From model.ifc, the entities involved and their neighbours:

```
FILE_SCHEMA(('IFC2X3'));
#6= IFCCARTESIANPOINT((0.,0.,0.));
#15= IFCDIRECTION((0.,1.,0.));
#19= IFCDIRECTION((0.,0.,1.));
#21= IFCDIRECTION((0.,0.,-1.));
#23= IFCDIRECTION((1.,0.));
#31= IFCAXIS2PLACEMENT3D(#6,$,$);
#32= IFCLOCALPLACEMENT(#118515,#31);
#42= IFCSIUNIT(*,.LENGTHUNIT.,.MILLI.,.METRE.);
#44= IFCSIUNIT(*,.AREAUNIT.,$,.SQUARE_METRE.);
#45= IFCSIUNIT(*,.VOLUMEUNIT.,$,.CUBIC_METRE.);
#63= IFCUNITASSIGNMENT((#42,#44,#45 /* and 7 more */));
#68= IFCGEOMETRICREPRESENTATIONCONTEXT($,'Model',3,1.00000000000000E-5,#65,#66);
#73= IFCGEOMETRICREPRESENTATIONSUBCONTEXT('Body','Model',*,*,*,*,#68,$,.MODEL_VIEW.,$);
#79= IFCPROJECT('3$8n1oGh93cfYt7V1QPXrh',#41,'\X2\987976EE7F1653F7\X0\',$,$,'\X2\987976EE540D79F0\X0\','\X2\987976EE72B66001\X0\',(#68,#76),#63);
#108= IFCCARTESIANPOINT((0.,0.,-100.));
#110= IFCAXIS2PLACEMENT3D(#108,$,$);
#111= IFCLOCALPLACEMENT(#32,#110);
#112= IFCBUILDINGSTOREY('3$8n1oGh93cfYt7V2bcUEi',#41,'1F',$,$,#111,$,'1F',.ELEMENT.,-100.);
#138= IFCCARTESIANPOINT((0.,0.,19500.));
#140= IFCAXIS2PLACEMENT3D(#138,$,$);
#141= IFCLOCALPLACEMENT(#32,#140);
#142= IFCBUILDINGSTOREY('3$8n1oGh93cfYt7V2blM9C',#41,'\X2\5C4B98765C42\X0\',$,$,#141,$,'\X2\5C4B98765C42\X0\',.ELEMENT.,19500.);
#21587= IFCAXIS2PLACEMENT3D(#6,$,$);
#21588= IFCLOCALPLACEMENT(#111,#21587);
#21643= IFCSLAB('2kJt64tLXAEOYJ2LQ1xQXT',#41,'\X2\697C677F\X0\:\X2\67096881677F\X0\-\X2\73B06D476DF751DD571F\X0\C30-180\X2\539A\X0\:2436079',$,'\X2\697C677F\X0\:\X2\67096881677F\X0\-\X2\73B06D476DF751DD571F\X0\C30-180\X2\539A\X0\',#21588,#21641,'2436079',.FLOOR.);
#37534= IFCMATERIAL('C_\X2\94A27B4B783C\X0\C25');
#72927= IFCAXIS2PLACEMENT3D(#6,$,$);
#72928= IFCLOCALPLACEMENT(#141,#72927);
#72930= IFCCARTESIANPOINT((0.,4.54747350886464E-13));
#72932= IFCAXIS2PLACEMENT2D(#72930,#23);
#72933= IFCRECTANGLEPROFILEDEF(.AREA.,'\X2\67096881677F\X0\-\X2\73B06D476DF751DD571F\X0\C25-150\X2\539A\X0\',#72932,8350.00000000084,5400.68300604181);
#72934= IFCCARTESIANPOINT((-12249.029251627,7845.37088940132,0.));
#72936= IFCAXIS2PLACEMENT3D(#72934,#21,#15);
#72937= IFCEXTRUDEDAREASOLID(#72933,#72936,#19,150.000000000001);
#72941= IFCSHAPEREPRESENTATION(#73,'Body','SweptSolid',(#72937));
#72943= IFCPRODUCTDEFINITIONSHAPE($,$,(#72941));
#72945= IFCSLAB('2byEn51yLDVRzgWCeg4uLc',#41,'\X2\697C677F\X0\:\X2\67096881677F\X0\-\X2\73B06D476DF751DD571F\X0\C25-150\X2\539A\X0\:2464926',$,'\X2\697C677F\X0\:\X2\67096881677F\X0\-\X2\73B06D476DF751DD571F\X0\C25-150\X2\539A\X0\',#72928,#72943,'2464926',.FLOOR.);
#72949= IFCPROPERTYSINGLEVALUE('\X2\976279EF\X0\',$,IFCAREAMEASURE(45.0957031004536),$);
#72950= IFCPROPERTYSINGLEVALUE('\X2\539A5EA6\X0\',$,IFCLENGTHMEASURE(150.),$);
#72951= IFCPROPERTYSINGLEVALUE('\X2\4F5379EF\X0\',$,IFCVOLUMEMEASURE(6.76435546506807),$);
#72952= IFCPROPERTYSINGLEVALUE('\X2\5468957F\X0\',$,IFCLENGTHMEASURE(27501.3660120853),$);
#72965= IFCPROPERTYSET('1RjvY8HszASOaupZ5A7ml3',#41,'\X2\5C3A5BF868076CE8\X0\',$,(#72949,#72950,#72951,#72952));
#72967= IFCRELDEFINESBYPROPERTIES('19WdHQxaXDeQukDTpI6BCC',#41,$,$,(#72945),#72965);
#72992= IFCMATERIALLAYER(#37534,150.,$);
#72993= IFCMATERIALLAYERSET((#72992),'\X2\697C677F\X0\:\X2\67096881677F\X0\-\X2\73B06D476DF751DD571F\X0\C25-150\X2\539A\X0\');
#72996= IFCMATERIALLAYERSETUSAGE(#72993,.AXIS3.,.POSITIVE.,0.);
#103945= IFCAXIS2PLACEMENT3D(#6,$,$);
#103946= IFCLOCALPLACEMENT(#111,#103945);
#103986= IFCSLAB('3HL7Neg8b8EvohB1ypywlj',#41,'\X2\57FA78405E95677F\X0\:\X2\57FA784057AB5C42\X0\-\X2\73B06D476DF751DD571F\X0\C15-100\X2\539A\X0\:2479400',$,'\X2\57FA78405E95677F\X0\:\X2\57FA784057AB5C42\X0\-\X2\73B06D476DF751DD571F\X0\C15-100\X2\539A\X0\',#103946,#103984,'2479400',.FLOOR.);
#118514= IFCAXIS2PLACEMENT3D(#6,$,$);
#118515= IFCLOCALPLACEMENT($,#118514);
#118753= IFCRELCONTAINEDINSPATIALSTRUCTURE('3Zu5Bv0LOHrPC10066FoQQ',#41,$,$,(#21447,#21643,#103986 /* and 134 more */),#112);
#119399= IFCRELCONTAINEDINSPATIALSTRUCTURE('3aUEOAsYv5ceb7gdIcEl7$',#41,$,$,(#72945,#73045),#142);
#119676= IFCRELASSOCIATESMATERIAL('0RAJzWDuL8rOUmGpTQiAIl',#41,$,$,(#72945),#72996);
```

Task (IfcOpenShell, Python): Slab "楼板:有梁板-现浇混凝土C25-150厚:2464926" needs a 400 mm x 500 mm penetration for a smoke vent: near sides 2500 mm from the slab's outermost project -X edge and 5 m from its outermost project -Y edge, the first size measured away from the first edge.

```python
import numpy as np
import ifcopenshell
import ifcopenshell.api.feature
import ifcopenshell.api.geometry
import ifcopenshell.api.pset
import ifcopenshell.api.root
import ifcopenshell.geom
import ifcopenshell.util.element
import ifcopenshell.util.placement
import ifcopenshell.util.representation
import ifcopenshell.util.shape
import ifcopenshell.util.unit

model = ifcopenshell.open("model.ifc")
unit_scale = ifcopenshell.util.unit.calculate_unit_scale(model)
area_scale = ifcopenshell.util.unit.calculate_unit_scale(model, "AREAUNIT")
volume_scale = ifcopenshell.util.unit.calculate_unit_scale(model, "VOLUMEUNIT")
settings = ifcopenshell.geom.settings()


def volume(element):
    """Net volume in cubic metres, openings subtracted."""
    shape = ifcopenshell.geom.create_shape(settings, element)
    return ifcopenshell.util.shape.get_volume(shape.geometry)


slab = model.by_guid("2byEn51yLDVRzgWCeg4uLc")
before = volume(slab)

# Extent in the slab's own axes, in metres. The edges named are its -X and -Y sides.
slab_shape = ifcopenshell.geom.create_shape(settings, slab)
vertices = ifcopenshell.util.shape.get_vertices(slab_shape.geometry)
x_min, y_min, bottom = vertices.min(axis=0)
top = vertices[:, 2].max()

opening = ifcopenshell.api.root.create_entity(model, ifc_class="IfcOpeningElement", name="Smoke vent opening")
context = ifcopenshell.util.representation.get_context(model, "Model", "Body", "MODEL_VIEW")
width, depth = 0.4, 0.5
outline = [(0.0, 0.0), (width, 0.0), (width, depth), (0.0, depth), (0.0, 0.0)]
# Overshoot both faces by 50 mm so the cut is clean.
shape = ifcopenshell.api.geometry.add_slab_representation(
    model, context=context, depth=top - bottom + 0.1, polyline=outline
)
ifcopenshell.api.geometry.assign_representation(model, product=opening, representation=shape)

matrix = ifcopenshell.util.placement.get_local_placement(slab.ObjectPlacement)
matrix[:, 3] = matrix @ np.append(np.array([x_min + 2.5, y_min + 5, bottom - 0.05]) / unit_scale, 1.0)
ifcopenshell.api.geometry.edit_object_placement(model, product=opening, matrix=matrix, is_si=False)
ifcopenshell.api.feature.add_feature(model, feature=opening, element=slab)

after = volume(slab)

# Update the slab's stored quantities.
pset = model.by_id(ifcopenshell.util.element.get_pset(slab, "尺寸标注", should_inherit=False)["id"])
ifcopenshell.api.pset.edit_pset(model, pset=pset, properties={
    "面积": model.create_entity("IfcAreaMeasure", after / (top - bottom) / area_scale),
    "体积": model.create_entity("IfcVolumeMeasure", after / volume_scale),
})

print(f"slab volume {before:.3f} -> {after:.3f} m3")

model.write("model_v2.ifc")
```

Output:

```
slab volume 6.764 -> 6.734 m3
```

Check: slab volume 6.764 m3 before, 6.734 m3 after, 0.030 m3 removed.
